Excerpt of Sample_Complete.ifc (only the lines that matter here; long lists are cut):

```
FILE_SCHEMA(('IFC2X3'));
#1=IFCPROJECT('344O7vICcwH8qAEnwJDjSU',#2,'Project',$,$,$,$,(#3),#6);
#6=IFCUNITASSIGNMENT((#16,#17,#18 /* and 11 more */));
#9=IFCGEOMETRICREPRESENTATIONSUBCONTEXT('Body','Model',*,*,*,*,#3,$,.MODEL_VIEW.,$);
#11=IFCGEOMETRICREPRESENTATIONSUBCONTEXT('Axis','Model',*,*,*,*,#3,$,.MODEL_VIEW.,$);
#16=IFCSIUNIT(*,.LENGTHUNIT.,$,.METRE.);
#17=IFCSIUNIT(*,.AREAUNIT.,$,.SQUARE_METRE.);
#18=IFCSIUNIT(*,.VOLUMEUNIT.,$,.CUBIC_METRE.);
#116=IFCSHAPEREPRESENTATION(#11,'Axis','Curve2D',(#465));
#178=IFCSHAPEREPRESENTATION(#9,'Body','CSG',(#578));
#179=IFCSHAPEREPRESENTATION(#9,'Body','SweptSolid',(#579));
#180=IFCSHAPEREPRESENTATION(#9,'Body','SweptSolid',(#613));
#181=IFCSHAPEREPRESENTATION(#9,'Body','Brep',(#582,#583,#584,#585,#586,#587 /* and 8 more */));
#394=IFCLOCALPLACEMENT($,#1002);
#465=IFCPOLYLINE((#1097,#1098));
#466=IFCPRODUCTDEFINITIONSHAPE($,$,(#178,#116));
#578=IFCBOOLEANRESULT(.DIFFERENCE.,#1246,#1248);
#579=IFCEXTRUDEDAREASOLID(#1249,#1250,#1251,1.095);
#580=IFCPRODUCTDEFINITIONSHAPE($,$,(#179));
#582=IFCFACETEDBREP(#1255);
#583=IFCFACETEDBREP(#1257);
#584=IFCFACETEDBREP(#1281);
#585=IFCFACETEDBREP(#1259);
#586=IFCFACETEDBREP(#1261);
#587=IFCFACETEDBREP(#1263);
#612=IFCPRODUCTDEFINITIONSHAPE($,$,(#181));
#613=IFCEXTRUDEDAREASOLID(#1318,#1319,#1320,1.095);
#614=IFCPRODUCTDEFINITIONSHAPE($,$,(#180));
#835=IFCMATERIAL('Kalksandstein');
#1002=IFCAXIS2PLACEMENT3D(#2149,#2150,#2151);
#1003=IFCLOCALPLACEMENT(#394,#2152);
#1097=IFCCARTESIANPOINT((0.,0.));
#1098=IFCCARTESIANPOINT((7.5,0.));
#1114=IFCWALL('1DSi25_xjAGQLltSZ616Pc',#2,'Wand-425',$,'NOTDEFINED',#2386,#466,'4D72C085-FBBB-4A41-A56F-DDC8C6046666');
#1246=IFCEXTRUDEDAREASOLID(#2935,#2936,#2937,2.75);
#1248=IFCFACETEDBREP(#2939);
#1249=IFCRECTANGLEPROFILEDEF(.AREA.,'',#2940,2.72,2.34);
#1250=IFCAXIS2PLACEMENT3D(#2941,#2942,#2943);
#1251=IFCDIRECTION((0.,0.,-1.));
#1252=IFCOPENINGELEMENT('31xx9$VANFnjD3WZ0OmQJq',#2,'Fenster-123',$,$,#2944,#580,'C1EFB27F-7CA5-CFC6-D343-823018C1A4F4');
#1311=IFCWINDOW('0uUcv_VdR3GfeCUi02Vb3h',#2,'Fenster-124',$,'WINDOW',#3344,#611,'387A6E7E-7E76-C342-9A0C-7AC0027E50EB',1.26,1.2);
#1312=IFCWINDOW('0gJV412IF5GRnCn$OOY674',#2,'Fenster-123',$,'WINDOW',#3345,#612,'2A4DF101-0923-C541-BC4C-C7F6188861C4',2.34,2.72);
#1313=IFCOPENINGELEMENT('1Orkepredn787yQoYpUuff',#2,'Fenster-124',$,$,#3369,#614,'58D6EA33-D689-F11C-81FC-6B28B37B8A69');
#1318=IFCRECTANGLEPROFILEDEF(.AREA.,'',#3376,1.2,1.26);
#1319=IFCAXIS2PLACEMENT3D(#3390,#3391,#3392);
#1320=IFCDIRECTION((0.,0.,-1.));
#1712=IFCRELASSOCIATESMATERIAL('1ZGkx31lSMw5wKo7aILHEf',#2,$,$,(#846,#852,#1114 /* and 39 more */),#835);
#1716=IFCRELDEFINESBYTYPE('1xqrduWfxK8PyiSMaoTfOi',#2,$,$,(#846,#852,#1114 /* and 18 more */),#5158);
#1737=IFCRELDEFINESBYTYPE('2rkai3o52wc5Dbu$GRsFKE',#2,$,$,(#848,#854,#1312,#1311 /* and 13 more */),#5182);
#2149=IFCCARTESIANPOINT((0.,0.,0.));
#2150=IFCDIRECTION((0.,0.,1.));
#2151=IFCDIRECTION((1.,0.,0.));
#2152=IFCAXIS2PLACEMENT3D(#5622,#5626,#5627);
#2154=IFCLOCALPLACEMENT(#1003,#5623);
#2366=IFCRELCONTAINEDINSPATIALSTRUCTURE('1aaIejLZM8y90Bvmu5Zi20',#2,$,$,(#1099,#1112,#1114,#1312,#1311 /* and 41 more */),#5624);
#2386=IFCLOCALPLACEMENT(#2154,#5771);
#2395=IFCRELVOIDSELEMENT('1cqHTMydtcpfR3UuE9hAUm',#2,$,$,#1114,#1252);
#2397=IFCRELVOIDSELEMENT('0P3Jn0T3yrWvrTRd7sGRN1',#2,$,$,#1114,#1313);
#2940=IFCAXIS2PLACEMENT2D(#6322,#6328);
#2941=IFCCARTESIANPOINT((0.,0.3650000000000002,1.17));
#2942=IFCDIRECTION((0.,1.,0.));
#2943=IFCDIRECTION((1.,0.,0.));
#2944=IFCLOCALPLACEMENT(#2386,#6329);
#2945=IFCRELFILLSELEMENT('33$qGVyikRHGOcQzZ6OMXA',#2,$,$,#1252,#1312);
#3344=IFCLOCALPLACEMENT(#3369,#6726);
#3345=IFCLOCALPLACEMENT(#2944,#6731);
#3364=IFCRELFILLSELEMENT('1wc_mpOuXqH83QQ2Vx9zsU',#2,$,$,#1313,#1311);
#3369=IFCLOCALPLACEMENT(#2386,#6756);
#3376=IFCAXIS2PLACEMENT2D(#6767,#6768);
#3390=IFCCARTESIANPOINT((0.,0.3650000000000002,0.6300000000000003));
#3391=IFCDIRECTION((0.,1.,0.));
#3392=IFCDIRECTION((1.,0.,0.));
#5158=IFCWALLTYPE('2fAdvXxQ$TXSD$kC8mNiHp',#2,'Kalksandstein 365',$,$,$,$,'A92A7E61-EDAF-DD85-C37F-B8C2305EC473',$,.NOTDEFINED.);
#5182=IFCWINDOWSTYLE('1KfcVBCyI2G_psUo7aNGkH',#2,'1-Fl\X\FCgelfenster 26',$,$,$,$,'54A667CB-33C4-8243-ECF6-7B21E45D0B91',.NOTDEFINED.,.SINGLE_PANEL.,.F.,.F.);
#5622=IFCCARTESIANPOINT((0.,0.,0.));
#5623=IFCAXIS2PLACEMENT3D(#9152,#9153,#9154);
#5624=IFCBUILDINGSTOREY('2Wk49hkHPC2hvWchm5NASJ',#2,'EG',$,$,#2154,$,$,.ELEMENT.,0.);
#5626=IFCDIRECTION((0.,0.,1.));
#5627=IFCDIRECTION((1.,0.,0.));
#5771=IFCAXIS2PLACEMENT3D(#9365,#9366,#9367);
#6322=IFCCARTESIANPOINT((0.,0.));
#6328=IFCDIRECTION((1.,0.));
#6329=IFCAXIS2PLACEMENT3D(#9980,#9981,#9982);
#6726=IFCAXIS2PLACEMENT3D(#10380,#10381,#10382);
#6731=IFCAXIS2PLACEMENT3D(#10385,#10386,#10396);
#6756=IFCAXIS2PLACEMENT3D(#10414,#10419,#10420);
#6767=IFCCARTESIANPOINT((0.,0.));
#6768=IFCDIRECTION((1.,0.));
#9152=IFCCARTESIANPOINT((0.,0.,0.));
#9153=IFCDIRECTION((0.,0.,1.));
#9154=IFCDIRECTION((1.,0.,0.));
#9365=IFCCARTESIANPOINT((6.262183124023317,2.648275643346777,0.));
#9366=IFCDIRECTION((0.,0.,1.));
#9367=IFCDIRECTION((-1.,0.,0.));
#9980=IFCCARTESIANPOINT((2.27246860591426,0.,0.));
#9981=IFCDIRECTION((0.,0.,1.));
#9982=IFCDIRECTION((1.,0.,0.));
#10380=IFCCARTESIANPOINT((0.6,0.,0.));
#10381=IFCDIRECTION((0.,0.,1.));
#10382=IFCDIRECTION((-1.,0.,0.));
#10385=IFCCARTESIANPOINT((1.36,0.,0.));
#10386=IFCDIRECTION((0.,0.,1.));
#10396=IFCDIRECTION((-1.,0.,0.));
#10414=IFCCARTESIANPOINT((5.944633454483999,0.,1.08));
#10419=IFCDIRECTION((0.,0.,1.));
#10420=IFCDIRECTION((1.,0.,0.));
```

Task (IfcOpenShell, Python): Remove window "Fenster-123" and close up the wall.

```python
import ifcopenshell
import ifcopenshell.api.feature
import ifcopenshell.api.root
import ifcopenshell.geom
import ifcopenshell.util.shape

model = ifcopenshell.open("Sample_Complete.ifc")
settings = ifcopenshell.geom.settings()


def volume(element):
    """Net volume in cubic metres, openings subtracted."""
    shape = ifcopenshell.geom.create_shape(settings, element)
    return ifcopenshell.util.shape.get_volume(shape.geometry)


window = model.by_guid("0gJV412IF5GRnCn$OOY674")
opening = window.FillsVoids[0].RelatingOpeningElement
wall = opening.VoidsElements[0].RelatingBuildingElement
before = volume(wall)

ifcopenshell.api.root.remove_product(model, product=window)
ifcopenshell.api.feature.remove_feature(model, feature=opening)

after = volume(wall)

print(f"wall volume {before:.3f} -> {after:.3f} m3")

model.write("Sample_Complete_edited.ifc")
```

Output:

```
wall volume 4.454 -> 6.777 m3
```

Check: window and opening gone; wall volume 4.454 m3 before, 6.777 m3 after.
